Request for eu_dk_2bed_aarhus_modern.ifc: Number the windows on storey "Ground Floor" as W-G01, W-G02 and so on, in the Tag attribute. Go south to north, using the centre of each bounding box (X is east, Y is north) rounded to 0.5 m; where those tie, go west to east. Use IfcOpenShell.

First a look at what the model holds.

```python
import ifcopenshell
import ifcopenshell.util.element
import ifcopenshell.util.placement

model = ifcopenshell.open("eu_dk_2bed_aarhus_modern.ifc")
print(model.schema)
storey = next(s for s in model.by_type("IfcBuildingStorey") if s.Name == "Ground Floor")
windows = [e for e in ifcopenshell.util.element.get_decomposition(storey) if e.is_a("IfcWindow")]
for e in sorted(windows, key=lambda e: e.id()):
    origin = ifcopenshell.util.placement.get_local_placement(e.ObjectPlacement)[:3, 3]
    print(e.id(), e.Tag, e.Name, origin.round(2) + 0.0, sep=" | ")
```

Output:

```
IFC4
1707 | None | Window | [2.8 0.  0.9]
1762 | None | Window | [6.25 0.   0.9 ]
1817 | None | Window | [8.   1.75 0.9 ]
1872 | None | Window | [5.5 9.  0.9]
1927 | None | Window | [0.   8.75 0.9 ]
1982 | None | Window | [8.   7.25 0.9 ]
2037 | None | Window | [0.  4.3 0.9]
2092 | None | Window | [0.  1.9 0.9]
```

```python
import ifcopenshell
import ifcopenshell.geom
import ifcopenshell.util.element
import ifcopenshell.util.shape

model = ifcopenshell.open("eu_dk_2bed_aarhus_modern.ifc")
settings = ifcopenshell.geom.settings()
settings.set("use-world-coords", True)


def centre(element):
    shape = ifcopenshell.geom.create_shape(settings, element)
    return ifcopenshell.util.shape.get_bbox_centroid(shape.geometry)


storey = next(s for s in model.by_type("IfcBuildingStorey") if s.Name == "Ground Floor")
windows = [e for e in ifcopenshell.util.element.get_decomposition(storey) if e.is_a("IfcWindow")]

# Insertion points can sit at a corner or the storey origin, so sort by the geometry (in metres).
centres = {e: centre(e) for e in windows}
windows.sort(key=lambda e: (round(centres[e][1] / 0.5), centres[e][0]))

for i, e in enumerate(windows, start=1):
    number = f"W-G{i:02d}"
    e.Tag = number
    print(e.id(), number)

model.write("eu_dk_2bed_aarhus_modern_updated.ifc")
```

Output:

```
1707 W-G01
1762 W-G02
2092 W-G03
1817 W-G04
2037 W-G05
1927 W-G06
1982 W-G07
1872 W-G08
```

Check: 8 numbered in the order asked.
